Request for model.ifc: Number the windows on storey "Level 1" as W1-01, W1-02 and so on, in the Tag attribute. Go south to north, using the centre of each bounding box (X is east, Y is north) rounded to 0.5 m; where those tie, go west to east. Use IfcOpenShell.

First a look at what the model holds.

```python
import ifcopenshell
import ifcopenshell.util.element
import ifcopenshell.util.placement

model = ifcopenshell.open("model.ifc")
print(model.schema)
storey = next(s for s in model.by_type("IfcBuildingStorey") if s.Name == "Level 1")
windows = [e for e in ifcopenshell.util.element.get_decomposition(storey) if e.is_a("IfcWindow")]
for e in sorted(windows, key=lambda e: e.id()):
    origin = ifcopenshell.util.placement.get_local_placement(e.ObjectPlacement)[:3, 3]
    print(e.id(), e.Tag, e.Name, origin.round(2) + 0.0, sep=" | ")
```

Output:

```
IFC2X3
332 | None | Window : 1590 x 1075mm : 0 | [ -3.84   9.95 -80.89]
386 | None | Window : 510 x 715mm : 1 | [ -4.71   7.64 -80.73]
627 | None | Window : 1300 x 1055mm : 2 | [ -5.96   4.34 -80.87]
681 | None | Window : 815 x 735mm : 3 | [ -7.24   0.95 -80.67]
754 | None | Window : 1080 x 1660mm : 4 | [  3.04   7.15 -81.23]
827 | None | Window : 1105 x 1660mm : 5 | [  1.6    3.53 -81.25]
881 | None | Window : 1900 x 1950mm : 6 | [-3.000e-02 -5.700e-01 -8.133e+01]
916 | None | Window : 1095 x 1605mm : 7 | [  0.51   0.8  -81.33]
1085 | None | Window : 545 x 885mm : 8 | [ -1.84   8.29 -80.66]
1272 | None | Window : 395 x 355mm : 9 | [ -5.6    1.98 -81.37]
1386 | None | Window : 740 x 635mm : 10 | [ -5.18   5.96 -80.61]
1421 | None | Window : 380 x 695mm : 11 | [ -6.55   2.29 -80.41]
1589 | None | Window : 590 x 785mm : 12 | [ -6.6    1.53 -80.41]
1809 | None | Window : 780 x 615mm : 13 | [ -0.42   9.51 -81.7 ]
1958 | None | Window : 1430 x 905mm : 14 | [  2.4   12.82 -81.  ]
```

```python
import ifcopenshell
import ifcopenshell.geom
import ifcopenshell.util.element
import ifcopenshell.util.shape

model = ifcopenshell.open("model.ifc")
settings = ifcopenshell.geom.settings()
settings.set("use-world-coords", True)


def centre(element):
    shape = ifcopenshell.geom.create_shape(settings, element)
    return ifcopenshell.util.shape.get_bbox_centroid(shape.geometry)


storey = next(s for s in model.by_type("IfcBuildingStorey") if s.Name == "Level 1")
windows = [e for e in ifcopenshell.util.element.get_decomposition(storey) if e.is_a("IfcWindow")]

# Insertion points can sit at a corner or the storey origin, so sort by the geometry (in metres).
centres = {e: centre(e) for e in windows}
windows.sort(key=lambda e: (round(centres[e][1] / 0.5), centres[e][0]))

for i, e in enumerate(windows, start=1):
    number = f"W1-{i:02d}"
    e.Tag = number
    print(e.id(), number)

model.write("model_v2.ifc")
```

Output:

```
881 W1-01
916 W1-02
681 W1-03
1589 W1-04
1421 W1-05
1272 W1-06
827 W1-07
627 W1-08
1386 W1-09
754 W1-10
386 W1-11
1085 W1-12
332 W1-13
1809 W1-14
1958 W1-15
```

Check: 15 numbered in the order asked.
